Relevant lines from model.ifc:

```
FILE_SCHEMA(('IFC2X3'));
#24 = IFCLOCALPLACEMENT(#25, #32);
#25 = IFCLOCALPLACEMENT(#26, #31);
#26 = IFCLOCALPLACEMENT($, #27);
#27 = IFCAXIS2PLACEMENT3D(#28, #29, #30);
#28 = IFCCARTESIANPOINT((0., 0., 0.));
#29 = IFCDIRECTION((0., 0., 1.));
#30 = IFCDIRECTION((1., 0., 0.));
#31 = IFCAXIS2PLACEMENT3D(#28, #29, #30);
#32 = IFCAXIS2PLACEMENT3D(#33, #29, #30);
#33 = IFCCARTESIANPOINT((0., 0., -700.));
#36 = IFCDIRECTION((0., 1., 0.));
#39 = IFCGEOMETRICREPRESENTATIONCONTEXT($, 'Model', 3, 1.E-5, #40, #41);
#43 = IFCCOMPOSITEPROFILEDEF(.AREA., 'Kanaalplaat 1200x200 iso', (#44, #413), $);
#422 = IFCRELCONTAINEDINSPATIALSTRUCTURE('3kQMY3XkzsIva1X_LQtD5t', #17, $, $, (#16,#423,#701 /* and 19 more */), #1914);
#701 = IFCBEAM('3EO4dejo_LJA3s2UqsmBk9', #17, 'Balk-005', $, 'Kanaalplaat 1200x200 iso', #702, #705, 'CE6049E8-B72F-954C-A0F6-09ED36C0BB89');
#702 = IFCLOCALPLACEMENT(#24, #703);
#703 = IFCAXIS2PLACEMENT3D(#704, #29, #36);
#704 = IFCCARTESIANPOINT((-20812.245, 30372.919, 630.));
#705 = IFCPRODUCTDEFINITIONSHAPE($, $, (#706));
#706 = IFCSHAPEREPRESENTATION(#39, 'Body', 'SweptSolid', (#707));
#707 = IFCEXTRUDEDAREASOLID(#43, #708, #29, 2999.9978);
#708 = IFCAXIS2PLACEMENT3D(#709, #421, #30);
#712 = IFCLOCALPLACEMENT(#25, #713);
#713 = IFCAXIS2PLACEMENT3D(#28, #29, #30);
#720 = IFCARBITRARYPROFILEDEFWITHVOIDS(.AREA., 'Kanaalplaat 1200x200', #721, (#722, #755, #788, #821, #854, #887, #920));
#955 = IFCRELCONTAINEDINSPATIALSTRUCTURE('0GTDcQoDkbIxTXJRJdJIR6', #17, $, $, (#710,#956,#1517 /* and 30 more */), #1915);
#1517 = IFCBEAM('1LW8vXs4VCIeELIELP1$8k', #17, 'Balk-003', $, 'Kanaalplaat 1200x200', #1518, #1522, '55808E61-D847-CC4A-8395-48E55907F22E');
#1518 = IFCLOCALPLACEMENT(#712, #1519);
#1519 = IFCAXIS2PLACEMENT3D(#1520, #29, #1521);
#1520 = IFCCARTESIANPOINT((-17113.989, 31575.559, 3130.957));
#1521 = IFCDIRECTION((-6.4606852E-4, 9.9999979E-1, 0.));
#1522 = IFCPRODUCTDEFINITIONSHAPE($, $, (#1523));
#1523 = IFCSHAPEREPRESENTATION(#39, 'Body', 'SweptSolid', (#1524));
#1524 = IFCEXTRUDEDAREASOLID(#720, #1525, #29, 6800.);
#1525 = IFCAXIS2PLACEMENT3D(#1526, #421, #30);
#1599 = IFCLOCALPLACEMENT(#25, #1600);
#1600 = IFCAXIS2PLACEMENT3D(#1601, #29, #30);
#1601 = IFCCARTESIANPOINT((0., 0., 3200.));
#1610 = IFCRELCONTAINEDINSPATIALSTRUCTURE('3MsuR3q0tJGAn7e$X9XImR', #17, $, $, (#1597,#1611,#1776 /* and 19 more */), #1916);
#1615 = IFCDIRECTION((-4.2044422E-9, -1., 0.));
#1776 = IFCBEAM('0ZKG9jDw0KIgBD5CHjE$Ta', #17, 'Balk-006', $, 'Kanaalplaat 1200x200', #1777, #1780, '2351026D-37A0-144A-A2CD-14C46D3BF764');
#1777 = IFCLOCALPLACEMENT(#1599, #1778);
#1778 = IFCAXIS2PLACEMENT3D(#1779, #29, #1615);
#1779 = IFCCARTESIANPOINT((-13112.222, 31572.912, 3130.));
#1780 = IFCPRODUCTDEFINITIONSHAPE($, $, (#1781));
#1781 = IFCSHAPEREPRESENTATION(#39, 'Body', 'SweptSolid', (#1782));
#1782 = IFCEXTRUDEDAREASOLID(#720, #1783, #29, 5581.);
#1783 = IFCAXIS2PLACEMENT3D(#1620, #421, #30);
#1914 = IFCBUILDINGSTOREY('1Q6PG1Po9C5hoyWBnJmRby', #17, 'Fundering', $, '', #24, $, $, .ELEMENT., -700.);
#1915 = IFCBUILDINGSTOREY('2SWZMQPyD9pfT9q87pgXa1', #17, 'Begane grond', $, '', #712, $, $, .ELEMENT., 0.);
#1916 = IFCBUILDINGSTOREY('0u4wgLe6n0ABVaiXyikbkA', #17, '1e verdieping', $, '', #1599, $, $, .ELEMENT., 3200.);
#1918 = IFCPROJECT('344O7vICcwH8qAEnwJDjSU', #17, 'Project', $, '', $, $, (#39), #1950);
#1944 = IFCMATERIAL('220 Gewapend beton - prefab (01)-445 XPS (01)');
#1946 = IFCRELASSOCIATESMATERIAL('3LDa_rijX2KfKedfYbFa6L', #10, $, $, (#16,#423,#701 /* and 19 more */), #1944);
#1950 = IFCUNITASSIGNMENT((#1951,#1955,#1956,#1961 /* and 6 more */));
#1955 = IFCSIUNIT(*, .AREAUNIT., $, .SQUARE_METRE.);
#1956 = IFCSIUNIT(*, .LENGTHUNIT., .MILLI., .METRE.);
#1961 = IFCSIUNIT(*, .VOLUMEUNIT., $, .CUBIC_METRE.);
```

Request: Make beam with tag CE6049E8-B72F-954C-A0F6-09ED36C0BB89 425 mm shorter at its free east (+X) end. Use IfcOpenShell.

```python
import ifcopenshell

model = ifcopenshell.open("model.ifc")

member = model.by_guid("3EO4dejo_LJA3s2UqsmBk9")
change = -425.0

# The extrusion runs towards the end named, so only its depth changes.
body = next(r for r in member.Representation.Representations if r.RepresentationIdentifier == "Body")
solid = body.Items[0]
old_length = solid.Depth
solid.Depth += change

print(f"length {old_length:g} -> {solid.Depth:g}")

model.write("model_v2.ifc")
```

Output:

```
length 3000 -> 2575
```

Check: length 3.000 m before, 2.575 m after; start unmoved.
